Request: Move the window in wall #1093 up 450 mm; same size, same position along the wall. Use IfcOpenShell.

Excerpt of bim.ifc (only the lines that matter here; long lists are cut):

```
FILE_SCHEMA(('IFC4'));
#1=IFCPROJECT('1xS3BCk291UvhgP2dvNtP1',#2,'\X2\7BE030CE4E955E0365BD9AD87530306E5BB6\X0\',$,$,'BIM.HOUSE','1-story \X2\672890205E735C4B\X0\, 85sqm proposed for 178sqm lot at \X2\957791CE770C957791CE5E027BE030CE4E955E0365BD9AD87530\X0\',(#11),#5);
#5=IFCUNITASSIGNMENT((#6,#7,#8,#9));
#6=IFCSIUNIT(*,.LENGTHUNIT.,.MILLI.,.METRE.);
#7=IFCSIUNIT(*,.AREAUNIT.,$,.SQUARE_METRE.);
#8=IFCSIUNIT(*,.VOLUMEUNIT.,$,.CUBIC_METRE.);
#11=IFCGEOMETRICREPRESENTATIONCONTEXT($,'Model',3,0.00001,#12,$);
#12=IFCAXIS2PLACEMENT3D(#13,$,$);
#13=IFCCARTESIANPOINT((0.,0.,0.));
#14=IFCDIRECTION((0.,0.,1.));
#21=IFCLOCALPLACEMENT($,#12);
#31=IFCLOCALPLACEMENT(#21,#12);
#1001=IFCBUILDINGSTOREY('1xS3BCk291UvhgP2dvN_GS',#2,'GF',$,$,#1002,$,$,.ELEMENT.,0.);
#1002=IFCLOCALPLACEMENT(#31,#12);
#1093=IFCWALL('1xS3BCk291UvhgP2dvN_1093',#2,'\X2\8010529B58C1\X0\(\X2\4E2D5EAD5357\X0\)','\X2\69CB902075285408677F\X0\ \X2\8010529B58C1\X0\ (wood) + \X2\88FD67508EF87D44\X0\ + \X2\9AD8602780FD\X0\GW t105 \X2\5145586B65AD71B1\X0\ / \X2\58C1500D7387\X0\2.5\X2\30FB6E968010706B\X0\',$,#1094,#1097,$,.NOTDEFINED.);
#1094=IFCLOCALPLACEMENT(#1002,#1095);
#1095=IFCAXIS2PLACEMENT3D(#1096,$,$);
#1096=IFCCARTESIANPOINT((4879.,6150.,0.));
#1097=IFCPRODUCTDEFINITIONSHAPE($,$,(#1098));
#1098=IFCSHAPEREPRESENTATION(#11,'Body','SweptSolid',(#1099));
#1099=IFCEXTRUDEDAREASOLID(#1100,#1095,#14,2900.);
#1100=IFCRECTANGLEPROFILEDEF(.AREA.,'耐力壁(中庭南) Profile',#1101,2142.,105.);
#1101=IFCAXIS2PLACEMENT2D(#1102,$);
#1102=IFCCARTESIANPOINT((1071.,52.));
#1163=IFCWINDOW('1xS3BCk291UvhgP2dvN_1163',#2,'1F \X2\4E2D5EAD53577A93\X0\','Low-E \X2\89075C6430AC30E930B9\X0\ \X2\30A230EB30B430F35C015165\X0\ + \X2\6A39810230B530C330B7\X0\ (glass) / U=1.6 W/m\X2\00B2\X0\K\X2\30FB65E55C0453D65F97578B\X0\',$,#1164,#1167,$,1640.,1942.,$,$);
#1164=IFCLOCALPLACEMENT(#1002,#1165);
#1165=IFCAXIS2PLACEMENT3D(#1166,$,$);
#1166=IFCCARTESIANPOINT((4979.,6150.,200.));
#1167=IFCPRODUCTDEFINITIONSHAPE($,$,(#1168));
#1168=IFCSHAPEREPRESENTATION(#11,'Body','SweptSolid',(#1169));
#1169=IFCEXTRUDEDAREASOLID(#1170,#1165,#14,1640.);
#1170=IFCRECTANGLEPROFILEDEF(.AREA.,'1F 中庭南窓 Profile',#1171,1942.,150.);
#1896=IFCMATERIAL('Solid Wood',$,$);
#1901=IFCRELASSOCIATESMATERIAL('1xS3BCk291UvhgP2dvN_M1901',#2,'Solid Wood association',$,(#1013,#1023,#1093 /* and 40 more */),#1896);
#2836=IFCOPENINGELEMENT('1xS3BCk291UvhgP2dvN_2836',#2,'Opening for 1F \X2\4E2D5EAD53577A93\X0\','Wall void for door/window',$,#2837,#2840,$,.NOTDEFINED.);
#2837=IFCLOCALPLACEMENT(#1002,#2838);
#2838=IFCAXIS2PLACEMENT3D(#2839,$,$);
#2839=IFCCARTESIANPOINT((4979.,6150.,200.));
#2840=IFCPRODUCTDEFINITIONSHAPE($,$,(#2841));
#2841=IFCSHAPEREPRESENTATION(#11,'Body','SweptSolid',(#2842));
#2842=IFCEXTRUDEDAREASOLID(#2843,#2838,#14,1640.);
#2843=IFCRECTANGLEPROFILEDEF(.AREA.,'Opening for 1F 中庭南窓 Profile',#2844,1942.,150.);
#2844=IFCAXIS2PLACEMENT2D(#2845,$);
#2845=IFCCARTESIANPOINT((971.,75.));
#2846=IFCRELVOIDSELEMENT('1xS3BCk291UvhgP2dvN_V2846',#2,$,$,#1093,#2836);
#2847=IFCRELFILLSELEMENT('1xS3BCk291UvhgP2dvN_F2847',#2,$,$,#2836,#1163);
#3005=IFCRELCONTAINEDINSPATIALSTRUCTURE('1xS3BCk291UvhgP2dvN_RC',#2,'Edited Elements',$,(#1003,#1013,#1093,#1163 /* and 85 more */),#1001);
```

```python
import numpy as np
import ifcopenshell
import ifcopenshell.api.geometry
import ifcopenshell.util.placement
import ifcopenshell.util.unit

model = ifcopenshell.open("bim.ifc")
unit_scale = ifcopenshell.util.unit.calculate_unit_scale(model)

window = model.by_guid("1xS3BCk291UvhgP2dvN_1163")
opening = window.FillsVoids[0].RelatingOpeningElement
dz = 0.45 / unit_scale

shift = np.array([0.0, 0.0, dz])
# The window is not placed relative to its opening, so move both.
for product in (opening, window):
    matrix = ifcopenshell.util.placement.get_local_placement(product.ObjectPlacement)
    matrix[:3, 3] += shift
    ifcopenshell.api.geometry.edit_object_placement(model, product=product, matrix=matrix, is_si=False)

print(f"moved by {dz * unit_scale:+.3f} m")

model.write("bim_edited.ifc")
```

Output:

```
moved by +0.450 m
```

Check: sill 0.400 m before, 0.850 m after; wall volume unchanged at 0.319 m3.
